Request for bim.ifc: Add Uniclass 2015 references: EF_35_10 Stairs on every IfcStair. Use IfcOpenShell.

First a look at what the model holds.

```python
import ifcopenshell

model = ifcopenshell.open("bim.ifc")
print(model.schema)
print("classifications:", [c.Name for c in model.by_type("IfcClassification")])
for ifc_class in ("IfcDoor", "IfcRoof", "IfcStair", "IfcWall", "IfcWindow"):
    print(ifc_class, len(model.by_type(ifc_class)))
```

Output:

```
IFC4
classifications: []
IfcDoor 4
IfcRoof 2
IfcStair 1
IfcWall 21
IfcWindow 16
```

```python
import ifcopenshell
import ifcopenshell.api.classification

model = ifcopenshell.open("bim.ifc")

system = ifcopenshell.api.classification.add_classification(model, classification="Uniclass 2015")

codes = {
    "IfcStair": ("EF_35_10", "Stairs"),
}
for ifc_class, (code, name) in codes.items():
    products = model.by_type(ifc_class)
    ifcopenshell.api.classification.add_reference(
        model, products=products, classification=system, identification=code, name=name
    )
    print(code, len(products))

model.write("bim-out.ifc")
```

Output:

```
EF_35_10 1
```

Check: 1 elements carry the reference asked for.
